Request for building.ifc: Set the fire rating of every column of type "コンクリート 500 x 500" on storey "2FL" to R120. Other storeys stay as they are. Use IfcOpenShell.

First a look at what the model holds.

```python
import ifcopenshell
import ifcopenshell.util.element

model = ifcopenshell.open("building.ifc")
print(model.schema)
storey = next(s for s in model.by_type("IfcBuildingStorey") if s.Name == "2FL")
columns = [e for e in ifcopenshell.util.element.get_decomposition(storey) if e.is_a("IfcColumn")]
seen = {}
for e in columns:
    element_type = ifcopenshell.util.element.get_type(e)
    key = (element_type.Name if element_type != e and element_type else None, ifcopenshell.util.element.get_pset(e, "Pset_ColumnCommon", "FireRating"))
    seen[key] = seen.get(key, 0) + 1
for (name, value), count in sorted(seen.items(), key=str):
    print(count, "x", name, "|", value)
```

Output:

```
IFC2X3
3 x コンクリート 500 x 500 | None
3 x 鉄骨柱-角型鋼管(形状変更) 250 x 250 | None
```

```python
import ifcopenshell
import ifcopenshell.api.pset
import ifcopenshell.util.element

model = ifcopenshell.open("building.ifc")

storey = next(s for s in model.by_type("IfcBuildingStorey") if s.Name == "2FL")
columns = [e for e in ifcopenshell.util.element.get_decomposition(storey) if e.is_a("IfcColumn")]

count = 0
for e in columns:
    element_type = ifcopenshell.util.element.get_type(e)
    if element_type in (None, e) or element_type.Name != "コンクリート 500 x 500":
        continue
    # add_pset returns the element's existing set when there is one.
    pset = ifcopenshell.api.pset.add_pset(model, product=e, name="Pset_ColumnCommon")
    ifcopenshell.api.pset.edit_pset(model, pset=pset, properties={"FireRating": "R120"})
    count += 1

print(count, "columns updated")

model.write("building_edited.ifc")
```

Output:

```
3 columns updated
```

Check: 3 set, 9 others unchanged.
